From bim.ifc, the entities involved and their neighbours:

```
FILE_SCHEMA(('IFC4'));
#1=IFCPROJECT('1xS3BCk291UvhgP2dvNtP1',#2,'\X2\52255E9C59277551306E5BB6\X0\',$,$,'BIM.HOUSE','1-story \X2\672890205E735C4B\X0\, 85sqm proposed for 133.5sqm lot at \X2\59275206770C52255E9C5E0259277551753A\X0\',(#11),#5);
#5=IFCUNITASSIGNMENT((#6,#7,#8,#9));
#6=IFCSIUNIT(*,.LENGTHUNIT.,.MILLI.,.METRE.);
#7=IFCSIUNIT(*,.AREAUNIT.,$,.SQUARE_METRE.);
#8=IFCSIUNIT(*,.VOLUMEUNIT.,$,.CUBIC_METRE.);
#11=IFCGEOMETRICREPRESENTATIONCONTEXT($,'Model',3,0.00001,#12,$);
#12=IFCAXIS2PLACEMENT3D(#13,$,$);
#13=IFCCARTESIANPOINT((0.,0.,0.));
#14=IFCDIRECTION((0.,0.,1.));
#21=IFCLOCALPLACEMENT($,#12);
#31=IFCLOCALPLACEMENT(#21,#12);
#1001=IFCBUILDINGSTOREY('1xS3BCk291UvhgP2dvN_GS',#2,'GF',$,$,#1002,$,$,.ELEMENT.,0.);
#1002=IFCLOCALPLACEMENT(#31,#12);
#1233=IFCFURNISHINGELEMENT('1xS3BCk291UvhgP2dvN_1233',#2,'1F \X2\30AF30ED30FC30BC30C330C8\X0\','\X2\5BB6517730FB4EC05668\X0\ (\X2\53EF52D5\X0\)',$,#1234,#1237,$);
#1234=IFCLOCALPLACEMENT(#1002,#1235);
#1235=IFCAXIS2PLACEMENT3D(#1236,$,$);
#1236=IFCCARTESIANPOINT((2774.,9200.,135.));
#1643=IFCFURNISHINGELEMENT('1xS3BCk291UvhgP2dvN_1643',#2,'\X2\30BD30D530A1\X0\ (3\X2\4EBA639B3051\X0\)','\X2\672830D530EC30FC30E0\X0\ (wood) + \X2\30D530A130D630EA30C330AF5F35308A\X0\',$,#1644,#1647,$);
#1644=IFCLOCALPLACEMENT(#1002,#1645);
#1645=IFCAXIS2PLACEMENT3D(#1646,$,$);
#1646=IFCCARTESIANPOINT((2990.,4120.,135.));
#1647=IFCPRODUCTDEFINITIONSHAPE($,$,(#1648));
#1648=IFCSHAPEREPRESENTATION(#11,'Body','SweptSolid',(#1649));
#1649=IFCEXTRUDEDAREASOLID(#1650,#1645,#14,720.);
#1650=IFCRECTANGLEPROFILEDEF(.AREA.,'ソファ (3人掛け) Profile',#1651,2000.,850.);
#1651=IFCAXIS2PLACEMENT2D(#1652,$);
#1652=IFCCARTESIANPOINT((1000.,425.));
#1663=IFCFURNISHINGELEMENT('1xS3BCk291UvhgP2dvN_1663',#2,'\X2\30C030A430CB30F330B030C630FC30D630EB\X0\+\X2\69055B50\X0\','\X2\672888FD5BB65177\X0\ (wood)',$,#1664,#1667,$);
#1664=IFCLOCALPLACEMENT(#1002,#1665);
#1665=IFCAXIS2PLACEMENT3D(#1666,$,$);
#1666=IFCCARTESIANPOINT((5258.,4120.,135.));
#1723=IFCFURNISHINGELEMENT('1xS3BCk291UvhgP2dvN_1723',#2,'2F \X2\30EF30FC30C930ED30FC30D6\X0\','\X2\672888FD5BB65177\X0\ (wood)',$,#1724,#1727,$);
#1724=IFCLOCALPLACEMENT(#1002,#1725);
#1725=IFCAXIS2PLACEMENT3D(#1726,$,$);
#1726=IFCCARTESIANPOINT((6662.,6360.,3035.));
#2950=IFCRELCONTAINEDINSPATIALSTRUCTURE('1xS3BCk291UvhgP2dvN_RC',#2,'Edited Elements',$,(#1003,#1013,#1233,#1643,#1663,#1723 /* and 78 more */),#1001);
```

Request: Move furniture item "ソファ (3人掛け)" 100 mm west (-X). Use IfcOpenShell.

```python
import ifcopenshell
import ifcopenshell.api.geometry
import ifcopenshell.util.placement

model = ifcopenshell.open("bim.ifc")

item = model.by_guid("1xS3BCk291UvhgP2dvN_1643")
matrix = ifcopenshell.util.placement.get_local_placement(item.ObjectPlacement)
matrix[0, 3] -= 100.0
ifcopenshell.api.geometry.edit_object_placement(model, product=item, matrix=matrix, is_si=False)

print(ifcopenshell.util.placement.get_local_placement(item.ObjectPlacement).round(3) + 0.0)

model.write("bim_rev.ifc")
```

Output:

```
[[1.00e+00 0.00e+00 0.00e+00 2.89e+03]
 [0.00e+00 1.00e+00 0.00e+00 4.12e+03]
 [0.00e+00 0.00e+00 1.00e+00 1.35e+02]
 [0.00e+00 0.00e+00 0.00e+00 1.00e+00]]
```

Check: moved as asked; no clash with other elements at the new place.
